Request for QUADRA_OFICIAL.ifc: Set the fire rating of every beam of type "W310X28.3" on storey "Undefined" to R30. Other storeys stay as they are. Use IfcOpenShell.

First a look at what the model holds.

```python
import ifcopenshell
import ifcopenshell.util.element

model = ifcopenshell.open("QUADRA_OFICIAL.ifc")
print(model.schema)
storey = next(s for s in model.by_type("IfcBuildingStorey") if s.Name == "Undefined")
beams = [e for e in ifcopenshell.util.element.get_decomposition(storey) if e.is_a("IfcBeam")]
seen = {}
for e in beams:
    element_type = ifcopenshell.util.element.get_type(e)
    key = (element_type.Name if element_type != e and element_type else None, ifcopenshell.util.element.get_pset(e, "Pset_BeamCommon", "FireRating"))
    seen[key] = seen.get(key, 0) + 1
for (name, value), count in sorted(seen.items(), key=str):
    print(count, "x", name, "|", value)
```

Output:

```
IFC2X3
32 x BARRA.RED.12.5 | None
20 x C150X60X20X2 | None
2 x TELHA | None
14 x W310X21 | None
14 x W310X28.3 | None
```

```python
import ifcopenshell
import ifcopenshell.api.pset
import ifcopenshell.util.element

model = ifcopenshell.open("QUADRA_OFICIAL.ifc")

storey = next(s for s in model.by_type("IfcBuildingStorey") if s.Name == "Undefined")
beams = [e for e in ifcopenshell.util.element.get_decomposition(storey) if e.is_a("IfcBeam")]

count = 0
for e in beams:
    element_type = ifcopenshell.util.element.get_type(e)
    if element_type in (None, e) or element_type.Name != "W310X28.3":
        continue
    found = ifcopenshell.util.element.get_pset(e, "Pset_BeamCommon", should_inherit=False)
    if found:
        pset = model.by_id(found["id"])
        if len(ifcopenshell.util.element.get_elements_by_pset(pset)) > 1:
            pset = ifcopenshell.api.pset.unshare_pset(model, products=[e], pset=pset)[0]
    else:
        pset = ifcopenshell.api.pset.add_pset(model, product=e, name="Pset_BeamCommon")
    ifcopenshell.api.pset.edit_pset(model, pset=pset, properties={"FireRating": "R30"})
    count += 1

print(count, "beams updated")

model.write("QUADRA_OFICIAL_v2.ifc")
```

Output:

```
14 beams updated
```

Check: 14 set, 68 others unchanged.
